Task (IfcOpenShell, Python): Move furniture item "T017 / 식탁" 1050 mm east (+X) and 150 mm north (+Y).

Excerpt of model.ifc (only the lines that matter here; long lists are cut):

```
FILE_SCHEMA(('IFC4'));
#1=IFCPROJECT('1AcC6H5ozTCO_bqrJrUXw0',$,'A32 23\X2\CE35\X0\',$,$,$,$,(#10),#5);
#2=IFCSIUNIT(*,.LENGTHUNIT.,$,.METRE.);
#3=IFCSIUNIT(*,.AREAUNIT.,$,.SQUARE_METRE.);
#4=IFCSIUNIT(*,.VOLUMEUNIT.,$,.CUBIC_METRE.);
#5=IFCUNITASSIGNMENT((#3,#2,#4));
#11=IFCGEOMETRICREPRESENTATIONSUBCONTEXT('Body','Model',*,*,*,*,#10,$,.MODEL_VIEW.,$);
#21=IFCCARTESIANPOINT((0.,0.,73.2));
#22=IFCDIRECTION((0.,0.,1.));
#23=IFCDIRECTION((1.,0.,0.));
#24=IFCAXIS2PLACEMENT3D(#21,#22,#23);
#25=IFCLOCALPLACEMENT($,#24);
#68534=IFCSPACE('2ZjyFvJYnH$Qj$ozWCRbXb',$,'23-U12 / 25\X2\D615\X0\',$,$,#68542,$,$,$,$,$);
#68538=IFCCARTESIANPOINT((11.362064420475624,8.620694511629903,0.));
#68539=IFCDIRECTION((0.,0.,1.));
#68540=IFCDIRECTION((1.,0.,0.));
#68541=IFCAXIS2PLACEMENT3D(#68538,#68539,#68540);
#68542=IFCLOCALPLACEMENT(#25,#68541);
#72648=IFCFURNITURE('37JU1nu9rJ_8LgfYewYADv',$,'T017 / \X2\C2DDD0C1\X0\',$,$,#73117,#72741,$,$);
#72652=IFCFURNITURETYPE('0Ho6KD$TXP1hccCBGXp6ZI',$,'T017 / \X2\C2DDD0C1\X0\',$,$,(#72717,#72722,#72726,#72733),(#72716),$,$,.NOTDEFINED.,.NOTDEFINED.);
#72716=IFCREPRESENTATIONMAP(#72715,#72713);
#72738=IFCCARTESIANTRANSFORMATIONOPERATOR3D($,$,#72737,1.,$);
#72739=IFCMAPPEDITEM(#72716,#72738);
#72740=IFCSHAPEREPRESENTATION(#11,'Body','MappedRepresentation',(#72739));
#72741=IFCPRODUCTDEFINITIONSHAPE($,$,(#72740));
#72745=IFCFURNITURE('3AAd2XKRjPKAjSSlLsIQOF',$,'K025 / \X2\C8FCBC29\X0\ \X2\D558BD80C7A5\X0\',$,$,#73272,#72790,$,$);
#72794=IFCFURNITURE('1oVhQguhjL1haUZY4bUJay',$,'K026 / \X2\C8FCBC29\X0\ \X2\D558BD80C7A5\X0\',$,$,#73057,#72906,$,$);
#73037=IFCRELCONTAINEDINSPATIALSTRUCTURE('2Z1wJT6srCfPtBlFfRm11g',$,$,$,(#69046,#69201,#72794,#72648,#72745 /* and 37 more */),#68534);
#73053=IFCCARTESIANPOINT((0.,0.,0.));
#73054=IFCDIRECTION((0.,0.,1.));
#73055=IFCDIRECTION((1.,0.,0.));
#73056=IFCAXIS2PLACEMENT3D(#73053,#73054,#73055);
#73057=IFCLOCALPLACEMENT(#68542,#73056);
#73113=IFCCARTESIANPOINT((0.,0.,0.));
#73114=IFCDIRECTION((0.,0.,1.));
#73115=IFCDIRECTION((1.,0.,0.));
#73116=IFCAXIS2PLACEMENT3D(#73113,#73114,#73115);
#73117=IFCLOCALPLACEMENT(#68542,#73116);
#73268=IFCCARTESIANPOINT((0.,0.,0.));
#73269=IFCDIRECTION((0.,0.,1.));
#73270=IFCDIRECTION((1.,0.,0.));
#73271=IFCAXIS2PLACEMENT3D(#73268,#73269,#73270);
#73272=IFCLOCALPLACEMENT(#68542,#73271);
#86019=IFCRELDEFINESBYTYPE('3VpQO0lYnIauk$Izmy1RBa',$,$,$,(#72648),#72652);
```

```python
import ifcopenshell
import ifcopenshell.api.geometry
import ifcopenshell.util.placement
import ifcopenshell.util.unit

model = ifcopenshell.open("model.ifc")
unit_scale = ifcopenshell.util.unit.calculate_unit_scale(model)

item = model.by_id(72648)
matrix = ifcopenshell.util.placement.get_local_placement(item.ObjectPlacement)
matrix[0, 3] += 1.05 / unit_scale
matrix[1, 3] += 0.15 / unit_scale
ifcopenshell.api.geometry.edit_object_placement(model, product=item, matrix=matrix, is_si=False)

print(ifcopenshell.util.placement.get_local_placement(item.ObjectPlacement).round(3) + 0.0)

model.write("model_edited.ifc")
```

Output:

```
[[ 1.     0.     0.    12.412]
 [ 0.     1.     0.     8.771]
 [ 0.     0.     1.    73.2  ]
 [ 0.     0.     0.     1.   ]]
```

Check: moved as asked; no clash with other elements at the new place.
